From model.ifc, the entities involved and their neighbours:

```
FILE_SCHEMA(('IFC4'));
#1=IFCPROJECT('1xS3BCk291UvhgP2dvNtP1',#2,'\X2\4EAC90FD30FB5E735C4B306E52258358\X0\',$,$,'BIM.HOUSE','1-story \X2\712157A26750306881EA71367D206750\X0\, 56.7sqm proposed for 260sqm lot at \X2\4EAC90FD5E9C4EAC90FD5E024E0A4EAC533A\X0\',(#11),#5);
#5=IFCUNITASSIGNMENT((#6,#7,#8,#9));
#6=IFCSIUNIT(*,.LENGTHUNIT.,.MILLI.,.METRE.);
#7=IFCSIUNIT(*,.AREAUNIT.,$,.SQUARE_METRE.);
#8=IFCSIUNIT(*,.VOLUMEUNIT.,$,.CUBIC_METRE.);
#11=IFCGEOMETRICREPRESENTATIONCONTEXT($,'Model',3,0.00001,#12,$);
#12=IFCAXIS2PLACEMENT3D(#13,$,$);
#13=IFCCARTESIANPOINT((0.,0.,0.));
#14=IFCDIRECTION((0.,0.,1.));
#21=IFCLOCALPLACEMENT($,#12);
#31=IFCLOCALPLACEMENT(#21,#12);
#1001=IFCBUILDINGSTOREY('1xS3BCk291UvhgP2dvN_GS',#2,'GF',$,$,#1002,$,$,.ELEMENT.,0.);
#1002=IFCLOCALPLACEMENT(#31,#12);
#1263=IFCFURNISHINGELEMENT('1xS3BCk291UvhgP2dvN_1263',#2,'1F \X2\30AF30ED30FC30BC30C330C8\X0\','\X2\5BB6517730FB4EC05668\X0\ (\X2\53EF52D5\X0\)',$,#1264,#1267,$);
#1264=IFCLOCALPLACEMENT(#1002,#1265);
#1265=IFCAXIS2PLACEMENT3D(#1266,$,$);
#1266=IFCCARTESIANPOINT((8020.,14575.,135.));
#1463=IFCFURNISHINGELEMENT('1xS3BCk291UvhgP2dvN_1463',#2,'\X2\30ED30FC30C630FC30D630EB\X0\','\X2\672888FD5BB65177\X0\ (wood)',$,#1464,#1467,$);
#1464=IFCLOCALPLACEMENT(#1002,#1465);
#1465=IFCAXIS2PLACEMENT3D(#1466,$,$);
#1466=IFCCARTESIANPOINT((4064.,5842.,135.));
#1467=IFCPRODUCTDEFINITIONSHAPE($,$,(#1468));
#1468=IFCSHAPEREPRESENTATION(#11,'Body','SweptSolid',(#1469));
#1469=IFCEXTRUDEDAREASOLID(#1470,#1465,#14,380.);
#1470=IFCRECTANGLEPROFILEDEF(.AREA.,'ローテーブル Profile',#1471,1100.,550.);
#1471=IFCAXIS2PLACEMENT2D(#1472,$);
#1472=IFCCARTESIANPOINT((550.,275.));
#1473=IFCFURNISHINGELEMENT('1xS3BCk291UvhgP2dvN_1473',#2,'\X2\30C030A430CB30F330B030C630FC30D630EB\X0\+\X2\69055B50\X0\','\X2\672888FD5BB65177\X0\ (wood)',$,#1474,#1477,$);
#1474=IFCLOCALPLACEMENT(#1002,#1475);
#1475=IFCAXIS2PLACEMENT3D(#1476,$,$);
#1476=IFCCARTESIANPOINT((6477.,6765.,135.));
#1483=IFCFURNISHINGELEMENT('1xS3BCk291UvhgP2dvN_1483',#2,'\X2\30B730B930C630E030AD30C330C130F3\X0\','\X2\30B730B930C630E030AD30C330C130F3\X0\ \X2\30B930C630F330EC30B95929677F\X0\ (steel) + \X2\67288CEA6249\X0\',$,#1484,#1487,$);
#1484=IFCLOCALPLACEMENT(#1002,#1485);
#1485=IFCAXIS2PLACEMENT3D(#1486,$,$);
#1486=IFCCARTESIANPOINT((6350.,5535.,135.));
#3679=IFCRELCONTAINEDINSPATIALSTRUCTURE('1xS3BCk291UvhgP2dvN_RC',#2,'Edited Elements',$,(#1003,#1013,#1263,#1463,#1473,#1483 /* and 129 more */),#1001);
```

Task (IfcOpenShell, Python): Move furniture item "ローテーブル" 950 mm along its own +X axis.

```python
import ifcopenshell
import ifcopenshell.api.geometry
import ifcopenshell.util.placement
import ifcopenshell.util.unit

model = ifcopenshell.open("model.ifc")
unit_scale = ifcopenshell.util.unit.calculate_unit_scale(model)

item = model.by_guid("1xS3BCk291UvhgP2dvN_1463")
matrix = ifcopenshell.util.placement.get_local_placement(item.ObjectPlacement)
matrix[:3, 3] += matrix[:3, 0] * 0.95 / unit_scale
ifcopenshell.api.geometry.edit_object_placement(model, product=item, matrix=matrix, is_si=False)

print(ifcopenshell.util.placement.get_local_placement(item.ObjectPlacement).round(3) + 0.0)

model.write("model_edited.ifc")
```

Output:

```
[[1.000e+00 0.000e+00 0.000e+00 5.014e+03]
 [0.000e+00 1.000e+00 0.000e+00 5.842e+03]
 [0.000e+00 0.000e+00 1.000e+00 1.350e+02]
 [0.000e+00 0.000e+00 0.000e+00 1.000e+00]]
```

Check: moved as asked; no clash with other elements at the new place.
